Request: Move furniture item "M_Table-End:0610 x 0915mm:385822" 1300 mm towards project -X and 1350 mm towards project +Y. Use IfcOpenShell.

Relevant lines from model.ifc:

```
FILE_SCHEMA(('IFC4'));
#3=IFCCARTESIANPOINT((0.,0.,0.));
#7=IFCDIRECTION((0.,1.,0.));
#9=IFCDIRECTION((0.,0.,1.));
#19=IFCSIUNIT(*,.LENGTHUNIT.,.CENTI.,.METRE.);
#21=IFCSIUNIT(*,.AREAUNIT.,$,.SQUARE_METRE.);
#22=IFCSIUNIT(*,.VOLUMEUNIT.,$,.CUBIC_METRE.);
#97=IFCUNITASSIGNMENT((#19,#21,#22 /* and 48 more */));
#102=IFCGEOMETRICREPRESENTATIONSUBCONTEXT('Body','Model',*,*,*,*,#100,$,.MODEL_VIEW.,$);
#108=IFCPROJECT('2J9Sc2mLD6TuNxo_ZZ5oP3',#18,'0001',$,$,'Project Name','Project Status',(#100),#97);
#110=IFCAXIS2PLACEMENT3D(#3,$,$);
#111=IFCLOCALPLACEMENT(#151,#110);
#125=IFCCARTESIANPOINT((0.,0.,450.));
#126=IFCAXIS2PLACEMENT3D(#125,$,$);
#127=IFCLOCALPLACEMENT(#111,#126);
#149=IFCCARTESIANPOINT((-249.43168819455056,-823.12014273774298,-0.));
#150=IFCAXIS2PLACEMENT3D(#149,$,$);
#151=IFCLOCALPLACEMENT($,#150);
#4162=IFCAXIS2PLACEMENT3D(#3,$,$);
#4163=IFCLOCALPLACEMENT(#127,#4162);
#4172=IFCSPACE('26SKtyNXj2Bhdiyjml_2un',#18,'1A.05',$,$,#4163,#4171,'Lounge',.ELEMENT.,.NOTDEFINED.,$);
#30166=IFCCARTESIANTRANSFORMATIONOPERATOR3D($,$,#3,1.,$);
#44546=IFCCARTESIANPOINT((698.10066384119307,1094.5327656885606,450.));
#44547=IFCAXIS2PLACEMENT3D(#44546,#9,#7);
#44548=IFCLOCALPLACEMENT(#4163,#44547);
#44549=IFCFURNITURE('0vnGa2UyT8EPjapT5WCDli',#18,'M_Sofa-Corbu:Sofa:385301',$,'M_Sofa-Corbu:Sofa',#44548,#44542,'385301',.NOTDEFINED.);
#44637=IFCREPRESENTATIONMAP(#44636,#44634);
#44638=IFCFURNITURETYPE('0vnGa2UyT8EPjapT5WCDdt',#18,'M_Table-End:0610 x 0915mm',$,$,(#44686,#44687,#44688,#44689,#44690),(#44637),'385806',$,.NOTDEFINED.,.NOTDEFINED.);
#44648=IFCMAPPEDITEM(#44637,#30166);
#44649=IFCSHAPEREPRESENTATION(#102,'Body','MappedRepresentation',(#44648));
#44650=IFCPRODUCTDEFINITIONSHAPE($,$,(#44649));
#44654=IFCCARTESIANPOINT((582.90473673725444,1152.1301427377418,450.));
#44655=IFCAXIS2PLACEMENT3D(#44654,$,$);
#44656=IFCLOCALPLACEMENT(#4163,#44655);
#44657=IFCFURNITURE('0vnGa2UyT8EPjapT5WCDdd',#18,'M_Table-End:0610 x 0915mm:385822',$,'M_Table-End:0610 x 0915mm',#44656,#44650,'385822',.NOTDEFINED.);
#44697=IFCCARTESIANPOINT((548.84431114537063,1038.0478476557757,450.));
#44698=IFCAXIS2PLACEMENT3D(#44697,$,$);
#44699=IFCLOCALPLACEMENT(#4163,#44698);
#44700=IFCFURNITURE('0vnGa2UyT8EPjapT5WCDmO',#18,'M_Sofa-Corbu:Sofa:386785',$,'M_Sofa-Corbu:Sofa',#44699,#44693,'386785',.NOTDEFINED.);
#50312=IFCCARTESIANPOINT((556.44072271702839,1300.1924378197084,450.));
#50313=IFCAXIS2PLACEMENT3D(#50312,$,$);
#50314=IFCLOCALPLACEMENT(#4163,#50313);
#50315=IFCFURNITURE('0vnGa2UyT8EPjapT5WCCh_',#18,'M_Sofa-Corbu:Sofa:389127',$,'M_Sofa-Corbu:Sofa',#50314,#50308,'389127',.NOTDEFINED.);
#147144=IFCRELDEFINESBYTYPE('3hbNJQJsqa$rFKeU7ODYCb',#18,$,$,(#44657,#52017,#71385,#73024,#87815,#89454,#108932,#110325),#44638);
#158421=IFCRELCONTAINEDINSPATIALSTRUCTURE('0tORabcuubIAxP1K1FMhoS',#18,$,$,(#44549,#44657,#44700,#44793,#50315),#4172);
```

```python
import ifcopenshell
import ifcopenshell.api.geometry
import ifcopenshell.util.placement
import ifcopenshell.util.unit

model = ifcopenshell.open("model.ifc")
unit_scale = ifcopenshell.util.unit.calculate_unit_scale(model)

item = model.by_guid("0vnGa2UyT8EPjapT5WCDdd")
matrix = ifcopenshell.util.placement.get_local_placement(item.ObjectPlacement)
matrix[0, 3] -= 1.3 / unit_scale
matrix[1, 3] += 1.35 / unit_scale
ifcopenshell.api.geometry.edit_object_placement(model, product=item, matrix=matrix, is_si=False)

print(ifcopenshell.util.placement.get_local_placement(item.ObjectPlacement).round(3) + 0.0)

model.write("model_rev.ifc")
```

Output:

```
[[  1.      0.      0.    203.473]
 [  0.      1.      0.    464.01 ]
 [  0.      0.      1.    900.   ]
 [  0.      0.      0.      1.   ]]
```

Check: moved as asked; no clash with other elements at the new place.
